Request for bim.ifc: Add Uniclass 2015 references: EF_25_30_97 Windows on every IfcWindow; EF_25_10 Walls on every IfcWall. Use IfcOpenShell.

First a look at what the model holds.

```python
import ifcopenshell

model = ifcopenshell.open("bim.ifc")
print(model.schema)
print("classifications:", [c.Name for c in model.by_type("IfcClassification")])
for ifc_class in ("IfcDoor", "IfcRoof", "IfcStair", "IfcWall", "IfcWindow"):
    print(ifc_class, len(model.by_type(ifc_class)))
```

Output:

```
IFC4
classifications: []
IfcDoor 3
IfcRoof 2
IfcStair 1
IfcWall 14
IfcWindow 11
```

```python
import ifcopenshell
import ifcopenshell.api.classification

model = ifcopenshell.open("bim.ifc")

system = ifcopenshell.api.classification.add_classification(model, classification="Uniclass 2015")

codes = {
    "IfcWindow": ("EF_25_30_97", "Windows"),
    "IfcWall": ("EF_25_10", "Walls"),
}
for ifc_class, (code, name) in codes.items():
    products = model.by_type(ifc_class)
    ifcopenshell.api.classification.add_reference(
        model, products=products, classification=system, identification=code, name=name
    )
    print(code, len(products))

model.write("bim_rev.ifc")
```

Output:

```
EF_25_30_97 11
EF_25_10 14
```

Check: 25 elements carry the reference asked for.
